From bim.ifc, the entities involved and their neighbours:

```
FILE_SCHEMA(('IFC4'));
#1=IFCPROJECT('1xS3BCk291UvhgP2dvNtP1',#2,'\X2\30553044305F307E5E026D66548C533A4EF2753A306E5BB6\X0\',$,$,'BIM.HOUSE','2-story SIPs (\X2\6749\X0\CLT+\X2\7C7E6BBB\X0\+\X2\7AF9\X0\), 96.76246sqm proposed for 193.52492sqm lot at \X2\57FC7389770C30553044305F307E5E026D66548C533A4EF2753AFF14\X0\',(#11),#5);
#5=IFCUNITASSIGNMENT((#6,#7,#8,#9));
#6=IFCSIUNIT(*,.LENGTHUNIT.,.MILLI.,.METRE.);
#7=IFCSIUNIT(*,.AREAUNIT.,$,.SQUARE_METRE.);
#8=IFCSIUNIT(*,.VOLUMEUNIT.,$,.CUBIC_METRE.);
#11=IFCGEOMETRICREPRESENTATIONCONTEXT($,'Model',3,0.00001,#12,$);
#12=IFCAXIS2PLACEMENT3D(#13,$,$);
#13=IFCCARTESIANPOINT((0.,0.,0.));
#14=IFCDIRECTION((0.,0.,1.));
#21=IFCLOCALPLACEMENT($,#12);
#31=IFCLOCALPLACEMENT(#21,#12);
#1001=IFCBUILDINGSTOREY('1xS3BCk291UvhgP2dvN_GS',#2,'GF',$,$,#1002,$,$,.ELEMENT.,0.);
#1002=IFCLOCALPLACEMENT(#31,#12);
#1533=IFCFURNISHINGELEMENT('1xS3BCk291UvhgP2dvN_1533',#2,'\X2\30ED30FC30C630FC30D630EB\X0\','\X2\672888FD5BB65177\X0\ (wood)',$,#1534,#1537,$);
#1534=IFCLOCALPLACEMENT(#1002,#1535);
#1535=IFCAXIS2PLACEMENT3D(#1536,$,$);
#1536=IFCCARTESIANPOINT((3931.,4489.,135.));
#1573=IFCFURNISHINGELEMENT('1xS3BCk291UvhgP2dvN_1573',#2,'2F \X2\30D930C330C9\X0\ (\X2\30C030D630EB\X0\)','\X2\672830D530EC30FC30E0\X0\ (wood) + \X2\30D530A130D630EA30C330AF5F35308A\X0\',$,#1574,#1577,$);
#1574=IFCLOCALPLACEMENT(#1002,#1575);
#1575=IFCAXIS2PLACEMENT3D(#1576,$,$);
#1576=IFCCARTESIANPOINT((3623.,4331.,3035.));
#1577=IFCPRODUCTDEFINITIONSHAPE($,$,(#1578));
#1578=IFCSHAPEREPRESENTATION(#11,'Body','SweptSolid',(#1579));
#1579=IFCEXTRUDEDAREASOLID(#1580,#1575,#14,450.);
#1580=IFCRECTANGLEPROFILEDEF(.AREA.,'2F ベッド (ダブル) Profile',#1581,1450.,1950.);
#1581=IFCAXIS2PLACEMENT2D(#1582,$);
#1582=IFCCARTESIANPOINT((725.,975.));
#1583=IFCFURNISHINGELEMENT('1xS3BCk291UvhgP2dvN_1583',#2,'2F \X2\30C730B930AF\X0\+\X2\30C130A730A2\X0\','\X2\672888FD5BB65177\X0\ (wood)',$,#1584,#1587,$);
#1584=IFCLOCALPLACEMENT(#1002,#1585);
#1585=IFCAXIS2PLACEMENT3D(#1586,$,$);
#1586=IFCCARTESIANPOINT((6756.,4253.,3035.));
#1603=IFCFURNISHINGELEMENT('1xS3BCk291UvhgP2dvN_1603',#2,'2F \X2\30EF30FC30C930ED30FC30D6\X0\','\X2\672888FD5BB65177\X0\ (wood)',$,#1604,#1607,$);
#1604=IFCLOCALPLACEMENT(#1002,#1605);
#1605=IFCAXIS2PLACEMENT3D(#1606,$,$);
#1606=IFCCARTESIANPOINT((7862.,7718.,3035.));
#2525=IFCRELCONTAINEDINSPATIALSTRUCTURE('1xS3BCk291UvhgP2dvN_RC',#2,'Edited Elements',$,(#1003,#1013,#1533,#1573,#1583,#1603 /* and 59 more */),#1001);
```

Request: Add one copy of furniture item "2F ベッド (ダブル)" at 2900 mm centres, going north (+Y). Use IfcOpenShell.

```python
import numpy as np
import ifcopenshell
import ifcopenshell.api.geometry
import ifcopenshell.api.root
import ifcopenshell.util.element
import ifcopenshell.util.placement
import ifcopenshell.util.unit

model = ifcopenshell.open("bim.ifc")
unit_scale = ifcopenshell.util.unit.calculate_unit_scale(model)


def reuse_history(source, copy):
    """copy_class also copies each property set's owner history, people and application; keep the originals."""
    for rel in copy.IsDefinedBy:
        if rel.is_a("IfcRelDefinesByProperties") and (history := rel.RelatingPropertyDefinition.OwnerHistory):
            rel.RelatingPropertyDefinition.OwnerHistory = source.OwnerHistory
            ifcopenshell.util.element.remove_deep2(model, history)


source = model.by_guid("1xS3BCk291UvhgP2dvN_1573")
base = ifcopenshell.util.placement.get_local_placement(source.ObjectPlacement)
step = np.array([0.0, 1.0, 0.0]) * 2.9 / unit_scale

for i in range(1, 2):
    copy = ifcopenshell.api.root.copy_class(model, product=source)
    copy.Representation = ifcopenshell.util.element.copy_deep(
        model, source.Representation, exclude=["IfcGeometricRepresentationContext", "IfcRepresentationMap"]
    )
    reuse_history(source, copy)
    matrix = base.copy()
    matrix[:3, 3] += i * step
    print("added at", matrix[:3, 3].round(3) + 0.0)
    ifcopenshell.api.geometry.edit_object_placement(model, product=copy, matrix=matrix, is_si=False)

model.write("bim_edited.ifc")
```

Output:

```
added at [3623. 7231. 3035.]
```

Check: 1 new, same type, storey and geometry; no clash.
